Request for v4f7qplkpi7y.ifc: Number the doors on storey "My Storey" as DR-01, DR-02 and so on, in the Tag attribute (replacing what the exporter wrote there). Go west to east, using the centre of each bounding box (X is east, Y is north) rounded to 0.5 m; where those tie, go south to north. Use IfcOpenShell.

First a look at what the model holds.

```python
import ifcopenshell
import ifcopenshell.util.element
import ifcopenshell.util.placement

model = ifcopenshell.open("v4f7qplkpi7y.ifc")
print(model.schema)
storey = next(s for s in model.by_type("IfcBuildingStorey") if s.Name == "My Storey")
doors = [e for e in ifcopenshell.util.element.get_decomposition(storey) if e.is_a("IfcDoor")]
for e in sorted(doors, key=lambda e: e.id()):
    origin = ifcopenshell.util.placement.get_local_placement(e.ObjectPlacement)[:3, 3]
    print(e.id(), e.Tag, e.Name, origin.round(2) + 0.0, sep=" | ")
```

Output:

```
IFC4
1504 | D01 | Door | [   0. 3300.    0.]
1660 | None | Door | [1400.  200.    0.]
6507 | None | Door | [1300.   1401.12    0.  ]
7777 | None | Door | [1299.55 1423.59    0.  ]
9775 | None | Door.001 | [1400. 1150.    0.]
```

```python
import ifcopenshell
import ifcopenshell.geom
import ifcopenshell.util.element
import ifcopenshell.util.shape

model = ifcopenshell.open("v4f7qplkpi7y.ifc")
settings = ifcopenshell.geom.settings()
settings.set("use-world-coords", True)


def centre(element):
    shape = ifcopenshell.geom.create_shape(settings, element)
    return ifcopenshell.util.shape.get_bbox_centroid(shape.geometry)


storey = next(s for s in model.by_type("IfcBuildingStorey") if s.Name == "My Storey")
doors = [e for e in ifcopenshell.util.element.get_decomposition(storey) if e.is_a("IfcDoor")]

# Insertion points can sit at a corner or the storey origin, so sort by the geometry (in metres).
centres = {e: centre(e) for e in doors}
doors.sort(key=lambda e: (round(centres[e][0] / 0.5), centres[e][1]))

for i, e in enumerate(doors, start=1):
    number = f"DR-{i:02d}"
    e.Tag = number
    print(e.id(), number)

model.write("v4f7qplkpi7y_rev.ifc")
```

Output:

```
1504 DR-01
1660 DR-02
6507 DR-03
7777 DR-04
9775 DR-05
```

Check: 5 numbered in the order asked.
